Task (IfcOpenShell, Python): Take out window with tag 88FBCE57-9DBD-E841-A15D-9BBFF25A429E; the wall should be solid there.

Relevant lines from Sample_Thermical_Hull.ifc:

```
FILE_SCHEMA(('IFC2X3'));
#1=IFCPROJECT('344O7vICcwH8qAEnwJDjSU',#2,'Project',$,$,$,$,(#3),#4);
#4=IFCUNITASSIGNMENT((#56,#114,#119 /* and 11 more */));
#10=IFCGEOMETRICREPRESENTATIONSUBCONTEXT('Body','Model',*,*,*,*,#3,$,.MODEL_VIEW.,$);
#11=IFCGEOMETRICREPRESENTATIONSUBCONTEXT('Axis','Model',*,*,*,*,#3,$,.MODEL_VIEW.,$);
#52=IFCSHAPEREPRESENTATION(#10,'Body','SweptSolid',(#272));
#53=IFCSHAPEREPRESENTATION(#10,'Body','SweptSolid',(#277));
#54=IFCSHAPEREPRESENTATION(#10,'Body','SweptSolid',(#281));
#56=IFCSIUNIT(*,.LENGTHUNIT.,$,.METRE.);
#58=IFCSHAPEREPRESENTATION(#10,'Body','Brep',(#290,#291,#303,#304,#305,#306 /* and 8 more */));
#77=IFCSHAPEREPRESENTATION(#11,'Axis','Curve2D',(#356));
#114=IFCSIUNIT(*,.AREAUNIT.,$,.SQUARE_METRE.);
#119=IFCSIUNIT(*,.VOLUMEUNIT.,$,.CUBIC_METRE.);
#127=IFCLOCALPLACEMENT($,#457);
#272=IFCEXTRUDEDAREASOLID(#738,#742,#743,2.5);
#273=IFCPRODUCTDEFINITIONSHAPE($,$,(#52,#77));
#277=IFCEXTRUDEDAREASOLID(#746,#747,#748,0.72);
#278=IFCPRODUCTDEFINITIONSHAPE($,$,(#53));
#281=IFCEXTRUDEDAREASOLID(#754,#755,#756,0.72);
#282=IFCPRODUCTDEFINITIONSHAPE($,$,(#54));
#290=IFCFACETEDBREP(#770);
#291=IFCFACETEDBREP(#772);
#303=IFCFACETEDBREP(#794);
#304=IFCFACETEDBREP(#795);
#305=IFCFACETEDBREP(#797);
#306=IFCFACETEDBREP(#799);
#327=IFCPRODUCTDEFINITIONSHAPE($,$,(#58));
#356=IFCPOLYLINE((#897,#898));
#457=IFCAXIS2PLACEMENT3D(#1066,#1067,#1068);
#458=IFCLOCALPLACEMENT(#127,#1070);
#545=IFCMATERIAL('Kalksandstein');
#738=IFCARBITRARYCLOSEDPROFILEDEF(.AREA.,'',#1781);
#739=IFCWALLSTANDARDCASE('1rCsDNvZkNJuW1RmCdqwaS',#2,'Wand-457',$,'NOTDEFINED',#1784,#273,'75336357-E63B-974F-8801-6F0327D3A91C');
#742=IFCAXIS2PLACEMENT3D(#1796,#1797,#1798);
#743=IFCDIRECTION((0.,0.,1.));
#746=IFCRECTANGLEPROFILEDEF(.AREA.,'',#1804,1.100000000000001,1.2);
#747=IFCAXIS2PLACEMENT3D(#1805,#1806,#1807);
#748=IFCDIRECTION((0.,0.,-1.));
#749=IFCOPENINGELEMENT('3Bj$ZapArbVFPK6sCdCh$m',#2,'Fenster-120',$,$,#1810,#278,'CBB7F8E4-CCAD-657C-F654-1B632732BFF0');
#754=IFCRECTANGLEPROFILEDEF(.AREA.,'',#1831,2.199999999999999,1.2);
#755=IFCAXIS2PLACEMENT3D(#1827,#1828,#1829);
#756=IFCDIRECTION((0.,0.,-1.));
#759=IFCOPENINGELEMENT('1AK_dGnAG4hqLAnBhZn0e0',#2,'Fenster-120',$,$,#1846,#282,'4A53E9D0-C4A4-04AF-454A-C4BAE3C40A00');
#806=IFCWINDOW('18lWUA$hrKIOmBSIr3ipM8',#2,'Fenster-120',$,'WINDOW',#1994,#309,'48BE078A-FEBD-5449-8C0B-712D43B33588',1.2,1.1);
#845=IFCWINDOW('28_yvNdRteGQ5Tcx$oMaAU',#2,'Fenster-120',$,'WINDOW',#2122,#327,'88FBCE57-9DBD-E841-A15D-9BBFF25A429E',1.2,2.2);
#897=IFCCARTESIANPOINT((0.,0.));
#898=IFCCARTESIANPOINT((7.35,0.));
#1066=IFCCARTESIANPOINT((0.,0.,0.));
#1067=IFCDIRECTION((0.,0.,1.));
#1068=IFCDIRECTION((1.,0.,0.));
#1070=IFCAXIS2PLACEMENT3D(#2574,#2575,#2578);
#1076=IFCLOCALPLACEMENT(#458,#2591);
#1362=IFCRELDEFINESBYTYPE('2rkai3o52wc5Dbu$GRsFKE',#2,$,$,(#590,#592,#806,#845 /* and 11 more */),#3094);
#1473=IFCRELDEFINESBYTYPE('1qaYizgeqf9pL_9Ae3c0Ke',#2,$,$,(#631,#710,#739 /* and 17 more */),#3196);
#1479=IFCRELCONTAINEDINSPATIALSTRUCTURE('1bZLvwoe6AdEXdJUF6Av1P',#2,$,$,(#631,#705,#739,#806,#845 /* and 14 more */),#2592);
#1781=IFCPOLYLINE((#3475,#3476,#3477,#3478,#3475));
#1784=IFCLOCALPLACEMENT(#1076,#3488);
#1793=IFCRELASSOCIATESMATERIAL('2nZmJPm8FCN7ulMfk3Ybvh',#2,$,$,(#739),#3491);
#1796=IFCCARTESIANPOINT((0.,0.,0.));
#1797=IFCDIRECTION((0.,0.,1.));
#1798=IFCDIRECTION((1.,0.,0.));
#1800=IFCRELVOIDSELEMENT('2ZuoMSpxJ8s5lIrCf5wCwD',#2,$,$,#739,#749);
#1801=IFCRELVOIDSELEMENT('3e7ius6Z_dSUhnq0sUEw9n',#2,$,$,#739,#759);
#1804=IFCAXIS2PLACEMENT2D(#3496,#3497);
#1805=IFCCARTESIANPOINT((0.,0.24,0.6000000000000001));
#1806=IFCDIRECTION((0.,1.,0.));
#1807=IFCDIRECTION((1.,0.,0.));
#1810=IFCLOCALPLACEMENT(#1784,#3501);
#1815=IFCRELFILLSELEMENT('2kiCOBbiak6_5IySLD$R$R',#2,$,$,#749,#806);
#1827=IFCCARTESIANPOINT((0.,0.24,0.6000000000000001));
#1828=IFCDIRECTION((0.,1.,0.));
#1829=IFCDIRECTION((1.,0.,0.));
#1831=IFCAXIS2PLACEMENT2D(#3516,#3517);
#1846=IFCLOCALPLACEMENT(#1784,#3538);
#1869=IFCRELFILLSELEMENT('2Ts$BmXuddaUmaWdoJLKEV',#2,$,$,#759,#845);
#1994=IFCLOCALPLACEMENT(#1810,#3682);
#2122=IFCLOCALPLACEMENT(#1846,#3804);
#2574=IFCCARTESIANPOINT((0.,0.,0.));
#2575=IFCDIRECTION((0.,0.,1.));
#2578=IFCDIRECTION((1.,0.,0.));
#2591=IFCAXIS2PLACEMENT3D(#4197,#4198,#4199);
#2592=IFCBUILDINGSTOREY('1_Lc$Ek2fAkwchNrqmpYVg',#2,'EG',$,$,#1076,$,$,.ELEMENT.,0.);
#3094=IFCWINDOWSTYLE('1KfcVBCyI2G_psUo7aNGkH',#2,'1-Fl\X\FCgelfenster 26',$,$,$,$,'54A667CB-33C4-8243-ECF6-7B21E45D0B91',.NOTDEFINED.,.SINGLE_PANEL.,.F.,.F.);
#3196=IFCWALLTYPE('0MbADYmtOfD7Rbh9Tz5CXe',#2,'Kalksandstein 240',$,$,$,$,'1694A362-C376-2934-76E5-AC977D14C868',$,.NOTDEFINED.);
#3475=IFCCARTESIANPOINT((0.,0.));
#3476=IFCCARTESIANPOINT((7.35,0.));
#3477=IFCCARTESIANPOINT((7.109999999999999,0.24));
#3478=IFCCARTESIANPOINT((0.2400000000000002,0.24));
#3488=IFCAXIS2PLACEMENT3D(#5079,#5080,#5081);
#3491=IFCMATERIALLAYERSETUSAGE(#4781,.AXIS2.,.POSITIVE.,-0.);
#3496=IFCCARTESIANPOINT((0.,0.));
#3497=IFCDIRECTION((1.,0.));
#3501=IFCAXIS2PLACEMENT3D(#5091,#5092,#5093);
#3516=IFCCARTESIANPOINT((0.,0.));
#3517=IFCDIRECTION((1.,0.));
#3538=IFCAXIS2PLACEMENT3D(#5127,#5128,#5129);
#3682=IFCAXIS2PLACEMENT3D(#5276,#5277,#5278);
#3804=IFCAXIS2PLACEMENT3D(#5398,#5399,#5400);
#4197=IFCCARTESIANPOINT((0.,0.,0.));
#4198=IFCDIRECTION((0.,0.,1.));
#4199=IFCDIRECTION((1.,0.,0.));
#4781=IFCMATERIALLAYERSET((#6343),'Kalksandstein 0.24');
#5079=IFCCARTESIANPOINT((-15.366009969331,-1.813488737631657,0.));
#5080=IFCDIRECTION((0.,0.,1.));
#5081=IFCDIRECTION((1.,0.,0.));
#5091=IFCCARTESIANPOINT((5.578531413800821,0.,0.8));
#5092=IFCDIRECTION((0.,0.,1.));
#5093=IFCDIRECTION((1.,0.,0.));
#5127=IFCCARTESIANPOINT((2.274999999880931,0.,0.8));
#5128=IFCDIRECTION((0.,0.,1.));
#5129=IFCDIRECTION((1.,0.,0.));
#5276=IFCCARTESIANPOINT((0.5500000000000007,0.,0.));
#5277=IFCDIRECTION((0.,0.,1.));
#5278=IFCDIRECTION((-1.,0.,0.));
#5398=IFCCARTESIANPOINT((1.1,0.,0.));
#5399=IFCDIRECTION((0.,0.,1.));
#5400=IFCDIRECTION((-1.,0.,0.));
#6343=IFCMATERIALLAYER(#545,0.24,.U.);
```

```python
import ifcopenshell
import ifcopenshell.api.feature
import ifcopenshell.api.root
import ifcopenshell.geom
import ifcopenshell.util.shape

model = ifcopenshell.open("Sample_Thermical_Hull.ifc")
settings = ifcopenshell.geom.settings()


def volume(element):
    """Net volume in cubic metres, openings subtracted."""
    shape = ifcopenshell.geom.create_shape(settings, element)
    return ifcopenshell.util.shape.get_volume(shape.geometry)


window = model.by_id(845)
opening = window.FillsVoids[0].RelatingOpeningElement
wall = opening.VoidsElements[0].RelatingBuildingElement
before = volume(wall)

ifcopenshell.api.root.remove_product(model, product=window)
ifcopenshell.api.feature.remove_feature(model, feature=opening)

after = volume(wall)

print(f"wall volume {before:.3f} -> {after:.3f} m3")

model.write("Sample_Thermical_Hull_updated.ifc")
```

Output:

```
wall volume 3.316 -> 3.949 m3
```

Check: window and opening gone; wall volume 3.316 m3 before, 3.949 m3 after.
